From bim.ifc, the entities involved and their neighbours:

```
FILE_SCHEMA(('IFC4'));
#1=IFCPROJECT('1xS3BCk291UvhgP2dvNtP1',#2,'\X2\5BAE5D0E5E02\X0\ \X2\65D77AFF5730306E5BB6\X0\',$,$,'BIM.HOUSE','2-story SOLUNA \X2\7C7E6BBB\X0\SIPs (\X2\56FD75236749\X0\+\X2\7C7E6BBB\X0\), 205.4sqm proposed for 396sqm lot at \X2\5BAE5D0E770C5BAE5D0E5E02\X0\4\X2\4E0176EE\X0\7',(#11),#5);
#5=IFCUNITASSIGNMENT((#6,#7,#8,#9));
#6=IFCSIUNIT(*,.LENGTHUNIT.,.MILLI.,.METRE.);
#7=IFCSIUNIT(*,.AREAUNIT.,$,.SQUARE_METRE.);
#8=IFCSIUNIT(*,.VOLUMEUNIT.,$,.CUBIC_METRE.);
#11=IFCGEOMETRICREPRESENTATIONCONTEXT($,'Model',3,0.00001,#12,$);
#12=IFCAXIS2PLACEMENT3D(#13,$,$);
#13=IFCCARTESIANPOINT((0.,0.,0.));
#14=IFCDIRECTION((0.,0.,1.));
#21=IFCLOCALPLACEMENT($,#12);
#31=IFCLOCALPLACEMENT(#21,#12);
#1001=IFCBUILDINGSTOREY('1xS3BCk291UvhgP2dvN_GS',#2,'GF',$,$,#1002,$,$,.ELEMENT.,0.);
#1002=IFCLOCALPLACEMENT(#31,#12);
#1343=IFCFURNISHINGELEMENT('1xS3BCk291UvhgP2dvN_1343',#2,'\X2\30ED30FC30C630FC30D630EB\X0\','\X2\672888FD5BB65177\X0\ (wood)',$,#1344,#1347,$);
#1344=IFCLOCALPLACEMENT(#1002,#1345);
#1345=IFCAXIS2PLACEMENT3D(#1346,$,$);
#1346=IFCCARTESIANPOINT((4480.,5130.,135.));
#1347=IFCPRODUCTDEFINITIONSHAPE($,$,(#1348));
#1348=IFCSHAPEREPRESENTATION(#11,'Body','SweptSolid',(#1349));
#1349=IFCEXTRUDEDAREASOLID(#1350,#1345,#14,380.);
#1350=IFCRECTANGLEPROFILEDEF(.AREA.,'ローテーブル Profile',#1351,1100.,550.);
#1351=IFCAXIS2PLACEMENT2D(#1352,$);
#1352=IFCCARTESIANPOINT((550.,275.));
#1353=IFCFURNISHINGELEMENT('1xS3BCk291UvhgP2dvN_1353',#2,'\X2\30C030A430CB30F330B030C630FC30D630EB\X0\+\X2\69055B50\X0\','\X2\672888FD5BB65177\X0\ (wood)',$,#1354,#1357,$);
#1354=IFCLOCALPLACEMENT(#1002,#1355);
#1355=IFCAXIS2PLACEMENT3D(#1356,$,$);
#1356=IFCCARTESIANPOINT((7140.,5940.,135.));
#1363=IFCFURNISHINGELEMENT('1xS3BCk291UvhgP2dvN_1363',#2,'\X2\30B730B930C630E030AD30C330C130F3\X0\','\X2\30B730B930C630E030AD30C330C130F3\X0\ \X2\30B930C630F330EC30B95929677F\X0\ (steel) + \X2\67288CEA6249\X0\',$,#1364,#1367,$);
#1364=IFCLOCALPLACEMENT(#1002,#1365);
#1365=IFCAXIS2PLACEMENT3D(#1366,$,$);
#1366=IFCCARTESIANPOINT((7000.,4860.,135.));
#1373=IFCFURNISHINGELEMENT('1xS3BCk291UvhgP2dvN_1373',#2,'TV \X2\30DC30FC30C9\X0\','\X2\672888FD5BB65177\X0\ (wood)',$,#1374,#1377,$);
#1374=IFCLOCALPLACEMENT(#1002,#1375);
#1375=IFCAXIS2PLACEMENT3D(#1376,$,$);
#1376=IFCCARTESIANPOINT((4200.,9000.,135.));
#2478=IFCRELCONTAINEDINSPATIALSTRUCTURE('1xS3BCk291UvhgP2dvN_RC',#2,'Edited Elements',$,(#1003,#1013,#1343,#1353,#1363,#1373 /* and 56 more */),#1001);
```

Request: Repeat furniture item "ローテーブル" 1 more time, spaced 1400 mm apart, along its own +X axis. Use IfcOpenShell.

```python
import ifcopenshell
import ifcopenshell.api.geometry
import ifcopenshell.api.root
import ifcopenshell.util.element
import ifcopenshell.util.placement

model = ifcopenshell.open("bim.ifc")


def reuse_history(source, copy):
    """copy_class also copies each property set's owner history, people and application; keep the originals."""
    for rel in copy.IsDefinedBy:
        if rel.is_a("IfcRelDefinesByProperties") and (history := rel.RelatingPropertyDefinition.OwnerHistory):
            rel.RelatingPropertyDefinition.OwnerHistory = source.OwnerHistory
            ifcopenshell.util.element.remove_deep2(model, history)


source = model.by_id(1343)
base = ifcopenshell.util.placement.get_local_placement(source.ObjectPlacement)
step = base[:3, 0] * 1400.0

for i in range(1, 2):
    copy = ifcopenshell.api.root.copy_class(model, product=source)
    copy.Representation = ifcopenshell.util.element.copy_deep(
        model, source.Representation, exclude=["IfcGeometricRepresentationContext", "IfcRepresentationMap"]
    )
    reuse_history(source, copy)
    matrix = base.copy()
    matrix[:3, 3] += i * step
    print("added at", matrix[:3, 3].round(3) + 0.0)
    ifcopenshell.api.geometry.edit_object_placement(model, product=copy, matrix=matrix, is_si=False)

model.write("bim_rev.ifc")
```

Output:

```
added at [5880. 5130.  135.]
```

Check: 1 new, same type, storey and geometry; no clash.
